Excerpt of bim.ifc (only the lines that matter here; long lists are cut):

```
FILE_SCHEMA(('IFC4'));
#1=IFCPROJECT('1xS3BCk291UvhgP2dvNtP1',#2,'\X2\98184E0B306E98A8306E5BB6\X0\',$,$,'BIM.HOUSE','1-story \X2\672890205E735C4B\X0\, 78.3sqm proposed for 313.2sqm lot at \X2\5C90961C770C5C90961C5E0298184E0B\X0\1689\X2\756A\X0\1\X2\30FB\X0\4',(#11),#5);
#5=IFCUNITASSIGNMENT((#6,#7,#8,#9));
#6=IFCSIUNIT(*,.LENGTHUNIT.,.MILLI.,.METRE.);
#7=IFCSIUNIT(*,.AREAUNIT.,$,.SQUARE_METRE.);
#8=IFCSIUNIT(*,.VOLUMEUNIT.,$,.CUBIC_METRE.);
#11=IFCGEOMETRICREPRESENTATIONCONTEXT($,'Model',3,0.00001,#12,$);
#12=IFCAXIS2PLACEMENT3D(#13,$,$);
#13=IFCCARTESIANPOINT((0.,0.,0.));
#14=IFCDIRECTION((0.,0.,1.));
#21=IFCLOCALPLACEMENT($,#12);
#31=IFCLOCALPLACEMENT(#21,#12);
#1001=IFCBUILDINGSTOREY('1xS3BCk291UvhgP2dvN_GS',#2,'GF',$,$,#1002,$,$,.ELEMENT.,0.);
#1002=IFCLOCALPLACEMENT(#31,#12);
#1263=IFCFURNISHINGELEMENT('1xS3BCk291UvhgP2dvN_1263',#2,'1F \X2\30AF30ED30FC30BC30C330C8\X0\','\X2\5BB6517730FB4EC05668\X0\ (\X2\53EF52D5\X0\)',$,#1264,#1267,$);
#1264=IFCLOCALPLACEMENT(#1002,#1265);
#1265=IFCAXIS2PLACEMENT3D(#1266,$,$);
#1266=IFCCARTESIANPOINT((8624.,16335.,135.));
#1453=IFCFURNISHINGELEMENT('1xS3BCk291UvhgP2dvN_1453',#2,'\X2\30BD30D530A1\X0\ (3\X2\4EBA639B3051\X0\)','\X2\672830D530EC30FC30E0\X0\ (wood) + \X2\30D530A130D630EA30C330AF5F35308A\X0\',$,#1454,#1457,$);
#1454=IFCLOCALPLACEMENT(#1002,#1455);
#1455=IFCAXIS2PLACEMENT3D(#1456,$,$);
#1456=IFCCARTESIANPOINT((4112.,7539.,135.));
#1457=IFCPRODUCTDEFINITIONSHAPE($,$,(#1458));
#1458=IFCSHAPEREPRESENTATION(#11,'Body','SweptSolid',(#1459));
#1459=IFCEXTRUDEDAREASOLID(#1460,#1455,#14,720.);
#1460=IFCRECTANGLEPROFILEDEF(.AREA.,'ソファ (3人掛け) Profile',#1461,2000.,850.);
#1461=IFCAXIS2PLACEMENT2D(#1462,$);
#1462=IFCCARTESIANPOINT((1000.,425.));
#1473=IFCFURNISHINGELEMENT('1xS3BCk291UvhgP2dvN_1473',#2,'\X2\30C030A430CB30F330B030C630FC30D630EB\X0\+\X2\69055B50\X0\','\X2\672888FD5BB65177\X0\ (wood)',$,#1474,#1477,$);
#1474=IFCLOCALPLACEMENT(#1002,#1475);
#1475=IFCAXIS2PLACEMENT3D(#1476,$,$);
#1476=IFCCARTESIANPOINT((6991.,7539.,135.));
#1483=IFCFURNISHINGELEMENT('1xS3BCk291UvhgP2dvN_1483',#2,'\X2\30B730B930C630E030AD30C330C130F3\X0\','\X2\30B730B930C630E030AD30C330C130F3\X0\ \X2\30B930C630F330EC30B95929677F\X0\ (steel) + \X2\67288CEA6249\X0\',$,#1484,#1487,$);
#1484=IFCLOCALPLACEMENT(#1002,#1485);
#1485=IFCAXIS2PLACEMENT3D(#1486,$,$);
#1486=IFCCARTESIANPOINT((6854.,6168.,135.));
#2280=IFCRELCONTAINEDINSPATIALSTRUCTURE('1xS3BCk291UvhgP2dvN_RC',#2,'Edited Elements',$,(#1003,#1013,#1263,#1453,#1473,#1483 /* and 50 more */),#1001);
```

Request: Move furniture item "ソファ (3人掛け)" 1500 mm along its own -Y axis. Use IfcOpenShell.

```python
import ifcopenshell
import ifcopenshell.api.geometry
import ifcopenshell.util.placement
import ifcopenshell.util.unit

model = ifcopenshell.open("bim.ifc")
unit_scale = ifcopenshell.util.unit.calculate_unit_scale(model)

item = model.by_guid("1xS3BCk291UvhgP2dvN_1453")
matrix = ifcopenshell.util.placement.get_local_placement(item.ObjectPlacement)
matrix[:3, 3] -= matrix[:3, 1] * 1.5 / unit_scale
ifcopenshell.api.geometry.edit_object_placement(model, product=item, matrix=matrix, is_si=False)

print(ifcopenshell.util.placement.get_local_placement(item.ObjectPlacement).round(3) + 0.0)

model.write("bim-out.ifc")
```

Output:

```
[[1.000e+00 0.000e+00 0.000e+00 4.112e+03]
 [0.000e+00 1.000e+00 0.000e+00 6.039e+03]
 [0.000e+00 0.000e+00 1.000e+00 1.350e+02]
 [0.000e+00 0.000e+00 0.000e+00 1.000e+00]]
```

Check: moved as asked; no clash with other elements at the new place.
